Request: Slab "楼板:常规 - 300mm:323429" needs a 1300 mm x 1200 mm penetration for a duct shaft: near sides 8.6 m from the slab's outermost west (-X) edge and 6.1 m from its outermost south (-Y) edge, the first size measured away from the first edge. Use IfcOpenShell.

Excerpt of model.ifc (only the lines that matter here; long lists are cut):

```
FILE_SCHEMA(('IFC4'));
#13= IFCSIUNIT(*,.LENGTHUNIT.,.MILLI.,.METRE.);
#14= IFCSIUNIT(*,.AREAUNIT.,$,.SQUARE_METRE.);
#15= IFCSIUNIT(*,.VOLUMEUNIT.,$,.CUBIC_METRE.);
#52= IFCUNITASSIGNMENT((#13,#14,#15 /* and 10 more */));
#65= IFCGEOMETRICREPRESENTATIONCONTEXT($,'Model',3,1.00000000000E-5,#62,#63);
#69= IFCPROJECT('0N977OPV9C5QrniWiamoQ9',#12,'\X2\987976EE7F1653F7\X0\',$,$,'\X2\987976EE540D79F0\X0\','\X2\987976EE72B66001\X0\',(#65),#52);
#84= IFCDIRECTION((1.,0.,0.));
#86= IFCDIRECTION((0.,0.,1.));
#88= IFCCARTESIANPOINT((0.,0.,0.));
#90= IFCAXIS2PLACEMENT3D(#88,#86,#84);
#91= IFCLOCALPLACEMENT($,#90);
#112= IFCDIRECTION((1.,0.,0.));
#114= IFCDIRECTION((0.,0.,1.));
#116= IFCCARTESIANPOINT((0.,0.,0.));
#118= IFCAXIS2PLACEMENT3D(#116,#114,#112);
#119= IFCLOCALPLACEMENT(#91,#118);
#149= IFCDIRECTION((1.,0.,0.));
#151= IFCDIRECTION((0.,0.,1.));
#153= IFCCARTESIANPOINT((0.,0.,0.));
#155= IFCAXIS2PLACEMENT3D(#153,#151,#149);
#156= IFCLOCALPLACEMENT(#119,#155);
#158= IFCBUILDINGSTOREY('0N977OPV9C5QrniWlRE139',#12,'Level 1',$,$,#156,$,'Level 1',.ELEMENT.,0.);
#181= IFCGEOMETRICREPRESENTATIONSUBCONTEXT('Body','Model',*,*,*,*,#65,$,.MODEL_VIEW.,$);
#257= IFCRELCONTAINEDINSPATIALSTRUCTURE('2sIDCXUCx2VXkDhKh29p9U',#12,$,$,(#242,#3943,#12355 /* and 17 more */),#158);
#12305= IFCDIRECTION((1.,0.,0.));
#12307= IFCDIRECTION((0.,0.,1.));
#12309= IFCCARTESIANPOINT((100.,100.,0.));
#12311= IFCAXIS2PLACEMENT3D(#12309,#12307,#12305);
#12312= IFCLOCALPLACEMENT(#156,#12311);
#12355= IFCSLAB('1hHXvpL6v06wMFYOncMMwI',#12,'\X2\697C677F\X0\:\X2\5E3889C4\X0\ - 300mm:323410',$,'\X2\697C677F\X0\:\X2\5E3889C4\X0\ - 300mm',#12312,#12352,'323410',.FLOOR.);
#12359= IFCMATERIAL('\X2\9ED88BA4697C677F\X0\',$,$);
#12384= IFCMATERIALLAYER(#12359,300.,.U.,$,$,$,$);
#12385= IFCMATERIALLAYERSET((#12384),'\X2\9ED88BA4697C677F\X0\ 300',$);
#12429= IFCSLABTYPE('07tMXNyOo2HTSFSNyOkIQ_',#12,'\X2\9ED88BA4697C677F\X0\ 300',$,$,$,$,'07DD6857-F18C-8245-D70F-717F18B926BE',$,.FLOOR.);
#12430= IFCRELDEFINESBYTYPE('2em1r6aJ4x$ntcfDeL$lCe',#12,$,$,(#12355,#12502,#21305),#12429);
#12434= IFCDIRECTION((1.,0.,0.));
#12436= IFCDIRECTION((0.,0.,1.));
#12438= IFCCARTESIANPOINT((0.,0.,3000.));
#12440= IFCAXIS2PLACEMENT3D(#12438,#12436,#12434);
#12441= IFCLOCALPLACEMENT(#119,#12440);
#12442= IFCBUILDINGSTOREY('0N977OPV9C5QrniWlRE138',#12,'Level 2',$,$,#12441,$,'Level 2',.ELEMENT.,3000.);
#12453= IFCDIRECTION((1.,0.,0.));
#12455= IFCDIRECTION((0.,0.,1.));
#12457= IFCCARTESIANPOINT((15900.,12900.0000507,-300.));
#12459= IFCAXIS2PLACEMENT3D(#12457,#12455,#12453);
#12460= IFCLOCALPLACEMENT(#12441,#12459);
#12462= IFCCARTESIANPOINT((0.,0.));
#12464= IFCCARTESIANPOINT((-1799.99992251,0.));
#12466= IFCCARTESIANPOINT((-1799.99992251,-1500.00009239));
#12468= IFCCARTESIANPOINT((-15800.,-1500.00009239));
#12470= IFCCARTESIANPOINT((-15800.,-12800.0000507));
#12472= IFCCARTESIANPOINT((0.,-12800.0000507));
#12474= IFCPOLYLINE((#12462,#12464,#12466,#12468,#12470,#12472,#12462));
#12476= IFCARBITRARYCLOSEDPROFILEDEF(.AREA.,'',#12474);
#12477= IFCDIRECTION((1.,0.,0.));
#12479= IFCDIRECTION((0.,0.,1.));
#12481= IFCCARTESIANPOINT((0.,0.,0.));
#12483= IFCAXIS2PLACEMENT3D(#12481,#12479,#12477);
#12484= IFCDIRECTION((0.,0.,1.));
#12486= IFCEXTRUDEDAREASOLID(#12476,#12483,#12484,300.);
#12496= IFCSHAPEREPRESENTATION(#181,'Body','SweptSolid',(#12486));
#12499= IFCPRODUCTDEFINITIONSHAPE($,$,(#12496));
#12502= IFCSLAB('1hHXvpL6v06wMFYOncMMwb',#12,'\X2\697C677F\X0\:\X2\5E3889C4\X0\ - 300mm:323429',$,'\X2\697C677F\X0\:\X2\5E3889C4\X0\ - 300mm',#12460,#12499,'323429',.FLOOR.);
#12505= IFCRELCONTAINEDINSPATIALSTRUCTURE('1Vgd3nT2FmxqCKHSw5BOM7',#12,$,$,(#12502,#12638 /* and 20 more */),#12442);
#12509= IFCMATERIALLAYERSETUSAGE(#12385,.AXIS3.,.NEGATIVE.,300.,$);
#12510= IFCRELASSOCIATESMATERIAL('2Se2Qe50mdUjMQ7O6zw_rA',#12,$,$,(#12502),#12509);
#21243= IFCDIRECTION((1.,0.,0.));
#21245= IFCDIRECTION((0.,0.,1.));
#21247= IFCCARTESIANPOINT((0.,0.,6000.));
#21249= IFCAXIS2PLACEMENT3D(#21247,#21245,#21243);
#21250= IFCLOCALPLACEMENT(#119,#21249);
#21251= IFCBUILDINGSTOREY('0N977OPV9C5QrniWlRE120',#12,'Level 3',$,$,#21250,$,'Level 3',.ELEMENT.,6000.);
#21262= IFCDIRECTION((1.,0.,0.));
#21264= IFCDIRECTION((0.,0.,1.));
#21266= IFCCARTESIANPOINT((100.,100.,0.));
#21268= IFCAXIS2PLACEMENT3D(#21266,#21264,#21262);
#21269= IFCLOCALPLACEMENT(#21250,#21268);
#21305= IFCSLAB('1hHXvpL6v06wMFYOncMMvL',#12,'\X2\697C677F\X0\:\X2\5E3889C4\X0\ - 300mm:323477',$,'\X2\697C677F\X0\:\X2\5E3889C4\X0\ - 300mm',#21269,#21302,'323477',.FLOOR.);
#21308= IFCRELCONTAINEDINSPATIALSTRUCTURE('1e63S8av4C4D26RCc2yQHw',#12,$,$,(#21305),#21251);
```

```python
import numpy as np
import ifcopenshell
import ifcopenshell.api.feature
import ifcopenshell.api.geometry
import ifcopenshell.api.root
import ifcopenshell.geom
import ifcopenshell.util.placement
import ifcopenshell.util.representation
import ifcopenshell.util.shape
import ifcopenshell.util.unit

model = ifcopenshell.open("model.ifc")
unit_scale = ifcopenshell.util.unit.calculate_unit_scale(model)
settings = ifcopenshell.geom.settings()


def volume(element):
    """Net volume in cubic metres, openings subtracted."""
    shape = ifcopenshell.geom.create_shape(settings, element)
    return ifcopenshell.util.shape.get_volume(shape.geometry)


slab = model.by_guid("1hHXvpL6v06wMFYOncMMwb")
before = volume(slab)

# Extent in the slab's own axes, in metres. The edges named are its -X and -Y sides.
slab_shape = ifcopenshell.geom.create_shape(settings, slab)
vertices = ifcopenshell.util.shape.get_vertices(slab_shape.geometry)
x_min, y_min, bottom = vertices.min(axis=0)
top = vertices[:, 2].max()

opening = ifcopenshell.api.root.create_entity(model, ifc_class="IfcOpeningElement", name="Duct shaft opening", predefined_type="OPENING")
context = ifcopenshell.util.representation.get_context(model, "Model", "Body", "MODEL_VIEW")
width, depth = 1.3, 1.2
outline = [(0.0, 0.0), (width, 0.0), (width, depth), (0.0, depth), (0.0, 0.0)]
# Overshoot both faces by 50 mm so the cut is clean.
shape = ifcopenshell.api.geometry.add_slab_representation(
    model, context=context, depth=top - bottom + 0.1, polyline=outline
)
ifcopenshell.api.geometry.assign_representation(model, product=opening, representation=shape)

matrix = ifcopenshell.util.placement.get_local_placement(slab.ObjectPlacement)
matrix[:, 3] = matrix @ np.append(np.array([x_min + 8.6, y_min + 6.1, bottom - 0.05]) / unit_scale, 1.0)
ifcopenshell.api.geometry.edit_object_placement(model, product=opening, matrix=matrix, is_si=False)
ifcopenshell.api.feature.add_feature(model, feature=opening, element=slab)

after = volume(slab)

print(f"slab volume {before:.3f} -> {after:.3f} m3")

model.write("model-out.ifc")
```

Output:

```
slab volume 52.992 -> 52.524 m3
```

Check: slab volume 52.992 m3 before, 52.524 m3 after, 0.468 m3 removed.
